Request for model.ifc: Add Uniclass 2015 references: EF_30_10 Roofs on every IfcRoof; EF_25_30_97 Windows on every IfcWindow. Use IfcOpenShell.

First a look at what the model holds.

```python
import ifcopenshell

model = ifcopenshell.open("model.ifc")
print(model.schema)
print("classifications:", [c.Name for c in model.by_type("IfcClassification")])
for ifc_class in ("IfcDoor", "IfcRoof", "IfcStair", "IfcWall", "IfcWindow"):
    print(ifc_class, len(model.by_type(ifc_class)))
```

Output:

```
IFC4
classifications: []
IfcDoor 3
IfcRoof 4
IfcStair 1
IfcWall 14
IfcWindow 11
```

```python
import ifcopenshell
import ifcopenshell.api.classification

model = ifcopenshell.open("model.ifc")

system = ifcopenshell.api.classification.add_classification(model, classification="Uniclass 2015")

codes = {
    "IfcRoof": ("EF_30_10", "Roofs"),
    "IfcWindow": ("EF_25_30_97", "Windows"),
}
for ifc_class, (code, name) in codes.items():
    products = model.by_type(ifc_class)
    ifcopenshell.api.classification.add_reference(
        model, products=products, classification=system, identification=code, name=name
    )
    print(code, len(products))

model.write("model_rev.ifc")
```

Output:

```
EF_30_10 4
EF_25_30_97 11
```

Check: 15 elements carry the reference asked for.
